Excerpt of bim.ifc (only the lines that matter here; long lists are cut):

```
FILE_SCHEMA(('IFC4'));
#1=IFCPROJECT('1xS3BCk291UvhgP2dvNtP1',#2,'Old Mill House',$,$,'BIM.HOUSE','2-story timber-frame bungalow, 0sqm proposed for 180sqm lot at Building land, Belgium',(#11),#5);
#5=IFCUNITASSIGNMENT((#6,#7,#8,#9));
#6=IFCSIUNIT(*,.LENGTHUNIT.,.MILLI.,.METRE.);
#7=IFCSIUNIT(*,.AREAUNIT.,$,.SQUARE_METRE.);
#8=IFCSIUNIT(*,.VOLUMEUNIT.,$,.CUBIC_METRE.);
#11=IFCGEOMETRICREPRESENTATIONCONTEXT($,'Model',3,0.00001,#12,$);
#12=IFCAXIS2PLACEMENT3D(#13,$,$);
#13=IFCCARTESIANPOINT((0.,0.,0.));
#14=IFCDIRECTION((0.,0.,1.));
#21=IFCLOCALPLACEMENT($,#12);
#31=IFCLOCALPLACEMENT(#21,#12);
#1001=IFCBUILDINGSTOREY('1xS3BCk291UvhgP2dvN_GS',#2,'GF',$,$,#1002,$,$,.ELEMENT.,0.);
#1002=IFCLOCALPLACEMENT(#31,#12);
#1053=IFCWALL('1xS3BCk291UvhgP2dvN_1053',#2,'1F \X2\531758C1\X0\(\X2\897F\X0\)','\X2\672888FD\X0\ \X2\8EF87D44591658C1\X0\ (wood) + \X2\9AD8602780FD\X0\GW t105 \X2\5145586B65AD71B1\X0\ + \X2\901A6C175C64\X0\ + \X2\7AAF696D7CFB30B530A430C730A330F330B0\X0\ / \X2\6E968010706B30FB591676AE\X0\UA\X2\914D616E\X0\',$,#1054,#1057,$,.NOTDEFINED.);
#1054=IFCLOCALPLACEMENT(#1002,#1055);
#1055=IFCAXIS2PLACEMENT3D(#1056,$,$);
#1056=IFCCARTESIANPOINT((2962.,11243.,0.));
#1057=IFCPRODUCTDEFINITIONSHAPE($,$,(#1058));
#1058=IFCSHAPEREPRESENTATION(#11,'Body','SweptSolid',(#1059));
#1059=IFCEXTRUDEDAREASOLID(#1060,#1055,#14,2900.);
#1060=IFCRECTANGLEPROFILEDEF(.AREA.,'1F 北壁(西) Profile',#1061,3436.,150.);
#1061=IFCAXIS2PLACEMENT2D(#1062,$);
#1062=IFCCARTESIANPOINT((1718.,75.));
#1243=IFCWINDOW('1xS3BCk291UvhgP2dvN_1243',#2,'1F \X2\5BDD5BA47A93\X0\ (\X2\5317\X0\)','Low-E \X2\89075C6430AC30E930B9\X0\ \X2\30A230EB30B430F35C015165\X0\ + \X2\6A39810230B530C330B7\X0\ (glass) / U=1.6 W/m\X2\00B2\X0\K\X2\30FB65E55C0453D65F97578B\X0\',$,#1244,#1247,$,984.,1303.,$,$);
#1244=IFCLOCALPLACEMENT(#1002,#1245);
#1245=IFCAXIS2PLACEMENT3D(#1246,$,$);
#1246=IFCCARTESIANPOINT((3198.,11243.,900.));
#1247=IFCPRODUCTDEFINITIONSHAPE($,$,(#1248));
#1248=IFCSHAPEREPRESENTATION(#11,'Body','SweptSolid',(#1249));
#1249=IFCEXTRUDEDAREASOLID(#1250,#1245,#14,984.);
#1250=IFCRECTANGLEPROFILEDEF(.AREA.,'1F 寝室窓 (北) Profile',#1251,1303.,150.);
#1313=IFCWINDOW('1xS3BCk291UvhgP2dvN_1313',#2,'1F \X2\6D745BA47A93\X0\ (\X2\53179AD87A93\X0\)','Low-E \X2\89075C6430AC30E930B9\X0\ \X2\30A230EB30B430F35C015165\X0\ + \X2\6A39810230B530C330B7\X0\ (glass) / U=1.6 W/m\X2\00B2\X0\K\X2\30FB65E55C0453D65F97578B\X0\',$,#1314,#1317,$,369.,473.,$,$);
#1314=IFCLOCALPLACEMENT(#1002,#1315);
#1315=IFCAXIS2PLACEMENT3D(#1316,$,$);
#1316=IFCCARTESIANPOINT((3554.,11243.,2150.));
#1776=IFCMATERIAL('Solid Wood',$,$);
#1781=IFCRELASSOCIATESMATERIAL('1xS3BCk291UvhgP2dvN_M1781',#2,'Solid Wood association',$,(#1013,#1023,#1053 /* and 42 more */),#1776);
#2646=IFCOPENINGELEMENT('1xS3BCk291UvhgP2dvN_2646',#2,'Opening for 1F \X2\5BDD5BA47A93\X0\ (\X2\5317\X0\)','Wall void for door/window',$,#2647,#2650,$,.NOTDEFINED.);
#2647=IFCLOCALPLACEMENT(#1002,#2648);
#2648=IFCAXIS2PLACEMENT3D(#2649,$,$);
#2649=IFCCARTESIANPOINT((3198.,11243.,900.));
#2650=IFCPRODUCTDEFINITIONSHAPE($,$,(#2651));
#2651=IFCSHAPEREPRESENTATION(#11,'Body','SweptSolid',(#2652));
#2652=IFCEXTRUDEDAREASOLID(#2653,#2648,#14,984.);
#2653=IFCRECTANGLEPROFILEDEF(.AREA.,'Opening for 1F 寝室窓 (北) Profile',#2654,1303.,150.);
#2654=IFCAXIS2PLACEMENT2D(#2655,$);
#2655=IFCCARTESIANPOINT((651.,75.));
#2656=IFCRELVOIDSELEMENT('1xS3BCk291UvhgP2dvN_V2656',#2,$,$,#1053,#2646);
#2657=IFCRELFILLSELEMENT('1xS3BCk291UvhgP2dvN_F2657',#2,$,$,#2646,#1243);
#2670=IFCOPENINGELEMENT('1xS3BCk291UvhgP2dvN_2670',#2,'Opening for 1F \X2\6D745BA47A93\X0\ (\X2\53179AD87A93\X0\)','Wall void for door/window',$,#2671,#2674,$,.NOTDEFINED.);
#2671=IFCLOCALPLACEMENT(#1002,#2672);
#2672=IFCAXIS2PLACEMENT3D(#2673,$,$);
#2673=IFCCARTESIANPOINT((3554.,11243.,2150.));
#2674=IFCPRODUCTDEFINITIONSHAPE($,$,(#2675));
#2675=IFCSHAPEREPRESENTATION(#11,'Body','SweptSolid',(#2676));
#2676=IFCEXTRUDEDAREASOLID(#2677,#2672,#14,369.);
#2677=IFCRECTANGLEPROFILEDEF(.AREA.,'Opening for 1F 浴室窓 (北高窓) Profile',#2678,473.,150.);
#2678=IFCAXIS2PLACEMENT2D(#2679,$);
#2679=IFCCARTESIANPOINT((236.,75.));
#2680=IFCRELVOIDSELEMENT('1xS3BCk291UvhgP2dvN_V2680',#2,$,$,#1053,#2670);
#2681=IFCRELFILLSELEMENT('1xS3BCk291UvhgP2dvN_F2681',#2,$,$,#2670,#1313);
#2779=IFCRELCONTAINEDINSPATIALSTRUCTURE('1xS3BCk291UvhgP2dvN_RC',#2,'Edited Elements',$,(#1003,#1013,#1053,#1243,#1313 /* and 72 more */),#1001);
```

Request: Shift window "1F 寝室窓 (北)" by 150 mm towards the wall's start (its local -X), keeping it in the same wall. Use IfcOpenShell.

```python
import ifcopenshell
import ifcopenshell.api.geometry
import ifcopenshell.util.placement
import ifcopenshell.util.unit

model = ifcopenshell.open("bim.ifc")
unit_scale = ifcopenshell.util.unit.calculate_unit_scale(model)

window = model.by_guid("1xS3BCk291UvhgP2dvN_1243")
opening = window.FillsVoids[0].RelatingOpeningElement
wall = opening.VoidsElements[0].RelatingBuildingElement

wall_matrix = ifcopenshell.util.placement.get_local_placement(wall.ObjectPlacement)
shift = wall_matrix[:3, 0] * -0.15 / unit_scale
before = ifcopenshell.util.placement.get_local_placement(window.ObjectPlacement)[:3, 3].copy()

# The window is not placed relative to its opening, so move both.
for product in (opening, window):
    matrix = ifcopenshell.util.placement.get_local_placement(product.ObjectPlacement)
    matrix[:3, 3] += shift
    ifcopenshell.api.geometry.edit_object_placement(model, product=product, matrix=matrix, is_si=False)

after = ifcopenshell.util.placement.get_local_placement(window.ObjectPlacement)[:3, 3]
print("window moved by", (after - before).round(3) + 0.0)

model.write("bim_updated.ifc")
```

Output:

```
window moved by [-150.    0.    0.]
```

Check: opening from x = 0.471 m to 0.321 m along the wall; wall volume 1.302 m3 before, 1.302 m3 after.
